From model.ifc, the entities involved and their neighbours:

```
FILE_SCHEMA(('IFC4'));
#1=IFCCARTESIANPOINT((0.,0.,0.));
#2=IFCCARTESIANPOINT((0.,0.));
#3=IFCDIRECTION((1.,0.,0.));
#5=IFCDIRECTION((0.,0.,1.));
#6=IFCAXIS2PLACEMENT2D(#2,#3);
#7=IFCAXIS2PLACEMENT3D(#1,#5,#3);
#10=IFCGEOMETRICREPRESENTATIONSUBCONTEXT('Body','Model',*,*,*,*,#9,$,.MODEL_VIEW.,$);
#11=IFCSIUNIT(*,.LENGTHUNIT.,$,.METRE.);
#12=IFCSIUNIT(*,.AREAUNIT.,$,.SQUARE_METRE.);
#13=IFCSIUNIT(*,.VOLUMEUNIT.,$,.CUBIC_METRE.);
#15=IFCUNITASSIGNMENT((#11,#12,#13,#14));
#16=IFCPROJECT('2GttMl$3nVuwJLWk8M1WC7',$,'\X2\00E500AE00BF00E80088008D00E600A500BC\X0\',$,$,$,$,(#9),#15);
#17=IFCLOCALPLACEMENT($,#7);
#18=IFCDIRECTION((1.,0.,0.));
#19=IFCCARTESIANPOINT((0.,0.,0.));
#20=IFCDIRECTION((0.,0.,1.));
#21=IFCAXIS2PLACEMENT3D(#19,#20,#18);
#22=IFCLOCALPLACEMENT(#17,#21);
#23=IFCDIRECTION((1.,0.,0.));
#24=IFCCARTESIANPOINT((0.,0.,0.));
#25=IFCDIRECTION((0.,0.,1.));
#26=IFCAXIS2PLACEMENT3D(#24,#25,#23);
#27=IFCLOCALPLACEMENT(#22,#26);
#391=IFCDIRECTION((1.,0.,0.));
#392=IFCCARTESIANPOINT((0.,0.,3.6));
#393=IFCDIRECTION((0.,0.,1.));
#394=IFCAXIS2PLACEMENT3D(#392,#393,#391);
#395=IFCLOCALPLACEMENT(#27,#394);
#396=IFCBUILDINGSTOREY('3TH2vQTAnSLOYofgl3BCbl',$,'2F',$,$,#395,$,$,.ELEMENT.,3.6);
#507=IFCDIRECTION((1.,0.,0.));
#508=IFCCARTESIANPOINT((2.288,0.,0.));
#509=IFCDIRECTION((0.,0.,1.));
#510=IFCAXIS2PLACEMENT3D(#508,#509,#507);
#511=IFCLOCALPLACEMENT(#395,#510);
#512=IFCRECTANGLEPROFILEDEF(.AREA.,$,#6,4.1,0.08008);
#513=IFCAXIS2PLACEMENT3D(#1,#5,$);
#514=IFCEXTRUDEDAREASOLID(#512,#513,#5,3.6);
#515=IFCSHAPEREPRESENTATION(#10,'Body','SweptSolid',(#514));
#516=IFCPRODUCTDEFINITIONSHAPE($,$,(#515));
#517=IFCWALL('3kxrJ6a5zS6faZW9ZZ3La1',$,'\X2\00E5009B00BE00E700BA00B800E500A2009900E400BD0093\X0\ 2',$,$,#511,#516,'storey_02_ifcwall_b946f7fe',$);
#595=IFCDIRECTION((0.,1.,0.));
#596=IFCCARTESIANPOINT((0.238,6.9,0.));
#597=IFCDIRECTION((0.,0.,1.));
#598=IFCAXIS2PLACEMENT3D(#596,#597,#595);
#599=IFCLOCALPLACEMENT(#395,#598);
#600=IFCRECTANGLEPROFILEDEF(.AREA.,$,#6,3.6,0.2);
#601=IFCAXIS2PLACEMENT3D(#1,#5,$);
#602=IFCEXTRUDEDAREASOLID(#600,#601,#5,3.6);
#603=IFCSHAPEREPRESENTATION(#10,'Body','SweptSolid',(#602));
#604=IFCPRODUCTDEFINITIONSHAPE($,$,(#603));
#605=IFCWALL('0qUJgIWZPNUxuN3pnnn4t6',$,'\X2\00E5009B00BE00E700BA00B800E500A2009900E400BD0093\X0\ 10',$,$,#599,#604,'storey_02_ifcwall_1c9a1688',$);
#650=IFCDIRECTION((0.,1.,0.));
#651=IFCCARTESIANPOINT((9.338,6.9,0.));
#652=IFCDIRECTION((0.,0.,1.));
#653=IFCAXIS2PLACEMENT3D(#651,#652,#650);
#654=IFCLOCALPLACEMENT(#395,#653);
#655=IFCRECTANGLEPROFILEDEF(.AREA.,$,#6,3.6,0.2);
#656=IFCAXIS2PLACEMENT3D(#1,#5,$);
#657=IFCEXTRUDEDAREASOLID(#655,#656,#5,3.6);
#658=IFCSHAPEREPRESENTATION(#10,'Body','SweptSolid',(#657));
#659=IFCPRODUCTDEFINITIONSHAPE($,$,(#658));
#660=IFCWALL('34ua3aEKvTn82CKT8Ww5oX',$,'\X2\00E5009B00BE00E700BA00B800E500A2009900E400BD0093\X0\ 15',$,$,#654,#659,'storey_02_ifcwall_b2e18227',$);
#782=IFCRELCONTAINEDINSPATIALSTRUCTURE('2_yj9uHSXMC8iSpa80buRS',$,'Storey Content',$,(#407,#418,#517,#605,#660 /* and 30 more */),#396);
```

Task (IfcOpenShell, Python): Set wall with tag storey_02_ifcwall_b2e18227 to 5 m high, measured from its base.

```python
import ifcopenshell
import ifcopenshell.geom
import ifcopenshell.util.representation
import ifcopenshell.util.shape

model = ifcopenshell.open("model.ifc")
settings = ifcopenshell.geom.settings()


def volume(element):
    """Net volume in cubic metres, openings subtracted."""
    shape = ifcopenshell.geom.create_shape(settings, element)
    return ifcopenshell.util.shape.get_volume(shape.geometry)


wall = model.by_id(660)
before = volume(wall)

body = ifcopenshell.util.representation.get_representation(wall, "Model", "Body")
solid = body.Items[0]
old_height = solid.Depth
solid.Depth = 5.0
after = volume(wall)

print(f"height {old_height:g} -> {solid.Depth:g}, volume {before:.3f} -> {after:.3f} m3")

model.write("model_updated.ifc")
```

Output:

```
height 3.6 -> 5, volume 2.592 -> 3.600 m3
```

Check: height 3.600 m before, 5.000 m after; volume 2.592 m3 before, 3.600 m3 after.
